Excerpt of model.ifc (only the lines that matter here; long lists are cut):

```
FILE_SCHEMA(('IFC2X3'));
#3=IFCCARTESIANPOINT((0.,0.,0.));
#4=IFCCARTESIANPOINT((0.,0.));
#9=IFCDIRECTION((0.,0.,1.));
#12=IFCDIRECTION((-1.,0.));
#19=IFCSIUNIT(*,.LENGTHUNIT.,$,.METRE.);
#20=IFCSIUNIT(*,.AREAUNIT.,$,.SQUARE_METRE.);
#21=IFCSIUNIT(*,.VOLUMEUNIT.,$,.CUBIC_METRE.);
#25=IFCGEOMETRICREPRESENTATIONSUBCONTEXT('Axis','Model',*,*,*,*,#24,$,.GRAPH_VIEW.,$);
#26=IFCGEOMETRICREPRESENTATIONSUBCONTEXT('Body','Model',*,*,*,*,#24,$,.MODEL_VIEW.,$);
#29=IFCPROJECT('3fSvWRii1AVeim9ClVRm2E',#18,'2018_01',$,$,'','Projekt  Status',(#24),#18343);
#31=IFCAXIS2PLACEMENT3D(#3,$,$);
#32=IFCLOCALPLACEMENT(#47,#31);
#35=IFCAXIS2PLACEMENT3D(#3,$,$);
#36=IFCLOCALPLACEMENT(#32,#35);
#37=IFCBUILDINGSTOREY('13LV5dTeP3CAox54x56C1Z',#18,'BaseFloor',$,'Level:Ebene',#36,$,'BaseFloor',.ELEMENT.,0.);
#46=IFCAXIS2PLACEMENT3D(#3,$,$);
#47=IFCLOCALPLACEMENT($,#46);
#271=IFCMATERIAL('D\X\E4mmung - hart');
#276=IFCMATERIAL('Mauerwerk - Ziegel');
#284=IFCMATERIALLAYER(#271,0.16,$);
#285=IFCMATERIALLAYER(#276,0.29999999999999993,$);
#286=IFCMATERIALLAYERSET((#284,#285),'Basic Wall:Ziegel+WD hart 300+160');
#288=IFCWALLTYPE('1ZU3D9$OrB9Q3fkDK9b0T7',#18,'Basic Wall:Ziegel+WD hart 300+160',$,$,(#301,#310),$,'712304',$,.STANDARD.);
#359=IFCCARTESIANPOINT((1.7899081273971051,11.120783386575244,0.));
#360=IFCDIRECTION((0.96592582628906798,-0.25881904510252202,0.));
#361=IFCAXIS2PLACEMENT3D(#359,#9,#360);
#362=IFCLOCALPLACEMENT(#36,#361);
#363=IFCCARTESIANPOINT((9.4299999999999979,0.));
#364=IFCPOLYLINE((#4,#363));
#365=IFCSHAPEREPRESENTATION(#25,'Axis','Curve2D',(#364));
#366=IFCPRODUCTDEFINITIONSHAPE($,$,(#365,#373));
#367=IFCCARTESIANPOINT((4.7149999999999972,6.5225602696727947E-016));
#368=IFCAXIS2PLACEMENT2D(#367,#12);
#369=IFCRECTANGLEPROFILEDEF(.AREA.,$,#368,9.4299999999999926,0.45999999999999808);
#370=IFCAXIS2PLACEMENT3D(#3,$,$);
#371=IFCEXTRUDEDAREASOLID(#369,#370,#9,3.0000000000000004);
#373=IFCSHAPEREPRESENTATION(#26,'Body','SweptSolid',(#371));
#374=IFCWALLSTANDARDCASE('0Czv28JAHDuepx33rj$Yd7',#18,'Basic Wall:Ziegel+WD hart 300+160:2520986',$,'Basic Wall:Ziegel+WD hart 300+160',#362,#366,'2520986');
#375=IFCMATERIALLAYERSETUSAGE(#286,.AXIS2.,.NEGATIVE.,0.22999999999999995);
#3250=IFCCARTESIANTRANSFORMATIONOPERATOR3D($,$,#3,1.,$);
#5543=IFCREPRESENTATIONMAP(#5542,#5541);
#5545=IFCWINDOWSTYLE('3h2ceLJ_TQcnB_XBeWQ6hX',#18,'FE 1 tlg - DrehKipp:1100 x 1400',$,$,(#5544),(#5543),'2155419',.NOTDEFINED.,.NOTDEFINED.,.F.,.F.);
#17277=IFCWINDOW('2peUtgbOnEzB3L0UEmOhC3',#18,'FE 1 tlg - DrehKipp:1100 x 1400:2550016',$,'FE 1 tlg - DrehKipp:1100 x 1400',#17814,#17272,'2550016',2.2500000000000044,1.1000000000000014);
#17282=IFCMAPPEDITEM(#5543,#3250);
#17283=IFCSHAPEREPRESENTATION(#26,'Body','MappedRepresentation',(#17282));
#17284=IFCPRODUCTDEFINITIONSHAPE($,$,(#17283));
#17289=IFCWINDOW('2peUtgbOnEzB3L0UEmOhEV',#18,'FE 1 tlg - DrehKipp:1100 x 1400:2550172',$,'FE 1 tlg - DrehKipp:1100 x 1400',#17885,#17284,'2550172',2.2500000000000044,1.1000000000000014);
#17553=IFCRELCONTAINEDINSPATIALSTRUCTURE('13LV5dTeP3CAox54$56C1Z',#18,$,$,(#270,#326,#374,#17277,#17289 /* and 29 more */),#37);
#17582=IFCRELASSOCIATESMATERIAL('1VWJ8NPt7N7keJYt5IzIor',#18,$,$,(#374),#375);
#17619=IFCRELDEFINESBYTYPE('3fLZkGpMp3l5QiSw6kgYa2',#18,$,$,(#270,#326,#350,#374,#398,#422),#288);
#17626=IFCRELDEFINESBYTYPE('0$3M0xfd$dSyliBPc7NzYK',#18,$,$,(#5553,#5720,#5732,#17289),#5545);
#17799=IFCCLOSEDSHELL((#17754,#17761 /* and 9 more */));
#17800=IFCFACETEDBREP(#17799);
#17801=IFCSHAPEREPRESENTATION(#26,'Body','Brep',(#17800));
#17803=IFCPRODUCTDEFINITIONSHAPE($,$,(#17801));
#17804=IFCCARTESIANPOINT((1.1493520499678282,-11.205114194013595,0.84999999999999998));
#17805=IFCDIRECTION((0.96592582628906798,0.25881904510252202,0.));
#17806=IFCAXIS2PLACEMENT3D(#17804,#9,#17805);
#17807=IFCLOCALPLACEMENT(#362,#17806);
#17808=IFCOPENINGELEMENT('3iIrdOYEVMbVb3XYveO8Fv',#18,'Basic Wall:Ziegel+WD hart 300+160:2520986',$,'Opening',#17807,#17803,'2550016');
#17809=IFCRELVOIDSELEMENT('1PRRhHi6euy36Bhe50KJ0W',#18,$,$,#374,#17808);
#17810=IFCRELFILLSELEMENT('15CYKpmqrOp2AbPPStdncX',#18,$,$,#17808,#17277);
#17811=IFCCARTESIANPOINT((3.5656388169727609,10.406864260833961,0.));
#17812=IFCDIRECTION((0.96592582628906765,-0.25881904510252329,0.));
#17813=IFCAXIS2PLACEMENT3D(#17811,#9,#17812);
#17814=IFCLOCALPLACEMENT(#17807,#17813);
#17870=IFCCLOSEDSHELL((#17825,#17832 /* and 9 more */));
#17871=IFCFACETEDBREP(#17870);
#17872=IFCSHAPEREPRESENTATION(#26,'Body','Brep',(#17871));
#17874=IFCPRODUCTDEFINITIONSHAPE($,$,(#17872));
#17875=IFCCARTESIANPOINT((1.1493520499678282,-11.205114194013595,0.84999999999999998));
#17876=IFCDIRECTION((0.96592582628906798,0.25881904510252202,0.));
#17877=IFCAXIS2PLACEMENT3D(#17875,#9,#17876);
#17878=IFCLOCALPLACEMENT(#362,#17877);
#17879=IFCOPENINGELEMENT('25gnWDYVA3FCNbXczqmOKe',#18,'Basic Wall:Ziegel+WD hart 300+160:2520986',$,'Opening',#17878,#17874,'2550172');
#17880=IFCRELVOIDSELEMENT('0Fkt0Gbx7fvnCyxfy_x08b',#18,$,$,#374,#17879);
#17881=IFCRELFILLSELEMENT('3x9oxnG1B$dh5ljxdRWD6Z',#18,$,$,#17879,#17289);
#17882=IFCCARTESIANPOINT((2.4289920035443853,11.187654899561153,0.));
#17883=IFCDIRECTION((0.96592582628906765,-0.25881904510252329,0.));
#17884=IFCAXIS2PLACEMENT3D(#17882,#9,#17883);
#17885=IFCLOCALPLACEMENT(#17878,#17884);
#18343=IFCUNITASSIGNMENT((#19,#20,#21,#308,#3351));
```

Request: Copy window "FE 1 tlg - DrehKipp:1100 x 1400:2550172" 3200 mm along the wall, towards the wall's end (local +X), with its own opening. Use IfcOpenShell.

```python
import ifcopenshell
import ifcopenshell.api.feature
import ifcopenshell.api.geometry
import ifcopenshell.api.root
import ifcopenshell.geom
import ifcopenshell.util.element
import ifcopenshell.util.placement
import ifcopenshell.util.shape
import ifcopenshell.util.unit

model = ifcopenshell.open("model.ifc")
unit_scale = ifcopenshell.util.unit.calculate_unit_scale(model)
settings = ifcopenshell.geom.settings()


def volume(element):
    """Net volume in cubic metres, openings subtracted."""
    shape = ifcopenshell.geom.create_shape(settings, element)
    return ifcopenshell.util.shape.get_volume(shape.geometry)


def reuse_history(source, copy):
    """copy_class also copies each property set's owner history, people and application; keep the originals."""
    for rel in copy.IsDefinedBy:
        if rel.is_a("IfcRelDefinesByProperties") and (history := rel.RelatingPropertyDefinition.OwnerHistory):
            rel.RelatingPropertyDefinition.OwnerHistory = source.OwnerHistory
            ifcopenshell.util.element.remove_deep2(model, history)


window = model.by_guid("2peUtgbOnEzB3L0UEmOhEV")
opening = window.FillsVoids[0].RelatingOpeningElement
wall = opening.VoidsElements[0].RelatingBuildingElement
before = volume(wall)
shift = ifcopenshell.util.placement.get_local_placement(wall.ObjectPlacement)[:3, 0] * 3.2 / unit_scale

# copy_class copies the void relationship, type, container and properties, but no geometry.
new_opening = ifcopenshell.api.root.copy_class(model, product=opening)
new_opening.Representation = ifcopenshell.util.element.copy_deep(
    model, opening.Representation, exclude=["IfcGeometricRepresentationContext", "IfcRepresentationMap"]
)
new_opening.Name = "Basic Wall:Ziegel+WD hart 300+160"
new_opening.Tag = None
new_window = ifcopenshell.api.root.copy_class(model, product=window)
new_window.Representation = ifcopenshell.util.element.copy_deep(
    model, window.Representation, exclude=["IfcGeometricRepresentationContext", "IfcRepresentationMap"]
)
new_window.Name = "FE 1 tlg - DrehKipp:1100 x 1400"
new_window.Tag = None
reuse_history(window, new_window)
fills = ifcopenshell.api.feature.add_filling(model, opening=new_opening, element=new_window)
fills.OwnerHistory = new_window.OwnerHistory  # required in IFC2X3

for old, new in ((opening, new_opening), (window, new_window)):
    matrix = ifcopenshell.util.placement.get_local_placement(old.ObjectPlacement)
    matrix[:3, 3] += shift
    ifcopenshell.api.geometry.edit_object_placement(model, product=new, matrix=matrix, is_si=False)

after = volume(wall)

print(f"wall volume {before:.3f} -> {after:.3f} m3")

model.write("model_updated.ifc")
```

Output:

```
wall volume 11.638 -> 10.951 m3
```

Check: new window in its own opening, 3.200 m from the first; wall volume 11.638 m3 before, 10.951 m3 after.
